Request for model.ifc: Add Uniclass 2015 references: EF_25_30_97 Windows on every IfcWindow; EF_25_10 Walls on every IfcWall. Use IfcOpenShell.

First a look at what the model holds.

```python
import ifcopenshell

model = ifcopenshell.open("model.ifc")
print(model.schema)
print("classifications:", [c.Name for c in model.by_type("IfcClassification")])
for ifc_class in ("IfcDoor", "IfcRoof", "IfcStair", "IfcWall", "IfcWindow"):
    print(ifc_class, len(model.by_type(ifc_class)))
```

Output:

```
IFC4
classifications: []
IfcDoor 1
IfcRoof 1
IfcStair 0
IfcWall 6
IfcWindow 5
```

```python
import ifcopenshell
import ifcopenshell.api.classification

model = ifcopenshell.open("model.ifc")

system = ifcopenshell.api.classification.add_classification(model, classification="Uniclass 2015")

codes = {
    "IfcWindow": ("EF_25_30_97", "Windows"),
    "IfcWall": ("EF_25_10", "Walls"),
}
for ifc_class, (code, name) in codes.items():
    products = model.by_type(ifc_class)
    ifcopenshell.api.classification.add_reference(
        model, products=products, classification=system, identification=code, name=name
    )
    print(code, len(products))

model.write("model_v2.ifc")
```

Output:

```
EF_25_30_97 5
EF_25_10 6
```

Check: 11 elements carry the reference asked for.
